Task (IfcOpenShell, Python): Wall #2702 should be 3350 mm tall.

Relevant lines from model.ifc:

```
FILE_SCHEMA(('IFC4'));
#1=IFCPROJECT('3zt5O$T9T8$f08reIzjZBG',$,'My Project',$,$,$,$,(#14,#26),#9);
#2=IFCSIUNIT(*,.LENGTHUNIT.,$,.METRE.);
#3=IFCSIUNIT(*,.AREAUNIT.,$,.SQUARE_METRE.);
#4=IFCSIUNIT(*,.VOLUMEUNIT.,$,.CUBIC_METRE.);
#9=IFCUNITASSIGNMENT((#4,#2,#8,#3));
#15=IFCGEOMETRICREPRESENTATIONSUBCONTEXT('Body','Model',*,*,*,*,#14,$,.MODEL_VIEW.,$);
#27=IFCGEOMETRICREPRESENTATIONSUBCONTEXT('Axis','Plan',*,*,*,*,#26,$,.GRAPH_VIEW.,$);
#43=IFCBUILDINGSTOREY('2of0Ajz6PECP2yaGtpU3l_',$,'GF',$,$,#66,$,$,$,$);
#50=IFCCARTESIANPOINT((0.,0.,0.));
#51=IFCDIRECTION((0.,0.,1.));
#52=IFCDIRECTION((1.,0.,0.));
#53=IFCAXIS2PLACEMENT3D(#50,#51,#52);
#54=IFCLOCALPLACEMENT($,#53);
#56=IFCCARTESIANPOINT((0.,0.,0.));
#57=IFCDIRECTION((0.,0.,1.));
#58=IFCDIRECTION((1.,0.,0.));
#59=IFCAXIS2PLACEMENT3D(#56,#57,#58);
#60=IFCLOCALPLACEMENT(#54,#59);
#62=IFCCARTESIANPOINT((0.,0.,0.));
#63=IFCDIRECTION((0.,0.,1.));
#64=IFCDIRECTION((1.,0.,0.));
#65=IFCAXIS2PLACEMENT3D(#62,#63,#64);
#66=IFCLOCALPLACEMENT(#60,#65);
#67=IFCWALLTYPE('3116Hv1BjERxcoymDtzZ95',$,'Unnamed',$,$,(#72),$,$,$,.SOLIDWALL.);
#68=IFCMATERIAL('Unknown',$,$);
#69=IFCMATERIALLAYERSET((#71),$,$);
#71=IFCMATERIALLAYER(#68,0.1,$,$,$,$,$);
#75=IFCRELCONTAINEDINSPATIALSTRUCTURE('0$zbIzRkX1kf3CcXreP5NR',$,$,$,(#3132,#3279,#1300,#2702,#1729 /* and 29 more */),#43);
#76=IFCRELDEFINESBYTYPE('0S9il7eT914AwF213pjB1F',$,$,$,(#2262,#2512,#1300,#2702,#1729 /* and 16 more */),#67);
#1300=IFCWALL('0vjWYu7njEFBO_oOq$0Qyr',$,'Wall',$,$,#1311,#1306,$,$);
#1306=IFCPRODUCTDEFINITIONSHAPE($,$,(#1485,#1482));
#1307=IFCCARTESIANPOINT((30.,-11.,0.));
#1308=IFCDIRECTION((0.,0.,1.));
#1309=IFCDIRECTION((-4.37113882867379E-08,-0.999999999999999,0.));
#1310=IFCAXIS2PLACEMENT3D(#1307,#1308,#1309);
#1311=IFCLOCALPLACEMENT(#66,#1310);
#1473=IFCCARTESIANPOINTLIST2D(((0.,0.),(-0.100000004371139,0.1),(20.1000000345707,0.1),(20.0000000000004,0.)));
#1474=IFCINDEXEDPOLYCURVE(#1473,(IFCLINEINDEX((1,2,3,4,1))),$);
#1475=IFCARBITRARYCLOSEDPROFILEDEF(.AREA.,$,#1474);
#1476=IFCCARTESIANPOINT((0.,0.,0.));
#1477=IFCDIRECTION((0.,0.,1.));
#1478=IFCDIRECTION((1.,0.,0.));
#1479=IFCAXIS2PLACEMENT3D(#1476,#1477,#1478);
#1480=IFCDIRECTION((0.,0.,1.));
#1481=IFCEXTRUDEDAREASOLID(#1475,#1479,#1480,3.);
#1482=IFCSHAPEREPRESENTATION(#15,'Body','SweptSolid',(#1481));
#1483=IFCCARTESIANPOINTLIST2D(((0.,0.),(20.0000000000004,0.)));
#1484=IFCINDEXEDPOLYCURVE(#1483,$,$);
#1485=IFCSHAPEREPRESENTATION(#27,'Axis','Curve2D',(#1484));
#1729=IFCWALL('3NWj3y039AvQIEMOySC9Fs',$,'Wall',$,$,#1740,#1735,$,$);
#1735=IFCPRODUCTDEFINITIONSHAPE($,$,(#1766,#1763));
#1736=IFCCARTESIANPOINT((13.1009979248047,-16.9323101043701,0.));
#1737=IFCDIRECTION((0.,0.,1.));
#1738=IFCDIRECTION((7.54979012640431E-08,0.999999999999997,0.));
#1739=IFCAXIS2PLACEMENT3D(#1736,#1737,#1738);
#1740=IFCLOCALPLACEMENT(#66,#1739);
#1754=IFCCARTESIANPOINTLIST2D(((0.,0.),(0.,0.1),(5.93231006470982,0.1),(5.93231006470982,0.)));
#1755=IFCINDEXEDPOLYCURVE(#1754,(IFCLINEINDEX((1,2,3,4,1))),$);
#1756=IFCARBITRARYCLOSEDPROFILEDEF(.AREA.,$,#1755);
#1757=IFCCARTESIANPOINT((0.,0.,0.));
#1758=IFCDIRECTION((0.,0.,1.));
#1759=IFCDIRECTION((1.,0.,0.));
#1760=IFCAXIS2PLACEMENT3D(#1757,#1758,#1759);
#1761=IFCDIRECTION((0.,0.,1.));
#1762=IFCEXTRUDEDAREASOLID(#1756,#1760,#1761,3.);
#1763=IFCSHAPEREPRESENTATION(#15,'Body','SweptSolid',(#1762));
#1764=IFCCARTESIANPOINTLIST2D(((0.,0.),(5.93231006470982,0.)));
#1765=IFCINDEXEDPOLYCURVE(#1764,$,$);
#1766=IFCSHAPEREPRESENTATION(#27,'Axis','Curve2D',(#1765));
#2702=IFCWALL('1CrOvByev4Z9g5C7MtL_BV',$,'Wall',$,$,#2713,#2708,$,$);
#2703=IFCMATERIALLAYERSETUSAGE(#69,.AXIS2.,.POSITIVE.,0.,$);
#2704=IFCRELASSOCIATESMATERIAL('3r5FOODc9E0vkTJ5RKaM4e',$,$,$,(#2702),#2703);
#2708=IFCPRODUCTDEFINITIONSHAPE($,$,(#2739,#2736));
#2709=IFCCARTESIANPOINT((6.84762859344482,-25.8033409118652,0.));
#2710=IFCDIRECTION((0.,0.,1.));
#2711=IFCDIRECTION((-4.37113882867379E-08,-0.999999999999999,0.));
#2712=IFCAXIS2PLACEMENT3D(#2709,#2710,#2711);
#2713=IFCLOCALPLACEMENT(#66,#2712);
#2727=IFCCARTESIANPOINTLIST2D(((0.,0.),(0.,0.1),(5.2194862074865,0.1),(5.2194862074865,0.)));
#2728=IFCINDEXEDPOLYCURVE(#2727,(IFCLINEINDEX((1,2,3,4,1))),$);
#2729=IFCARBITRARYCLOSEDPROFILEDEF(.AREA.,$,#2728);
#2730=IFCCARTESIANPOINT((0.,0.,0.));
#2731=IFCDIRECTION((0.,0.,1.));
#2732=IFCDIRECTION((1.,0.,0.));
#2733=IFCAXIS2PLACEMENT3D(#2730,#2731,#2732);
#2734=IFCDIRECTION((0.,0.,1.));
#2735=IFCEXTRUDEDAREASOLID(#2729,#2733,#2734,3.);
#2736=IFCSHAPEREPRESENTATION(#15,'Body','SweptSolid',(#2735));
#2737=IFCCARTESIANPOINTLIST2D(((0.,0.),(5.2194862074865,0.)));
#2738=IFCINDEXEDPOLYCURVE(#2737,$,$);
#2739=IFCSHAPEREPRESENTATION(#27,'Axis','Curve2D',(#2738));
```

```python
import ifcopenshell
import ifcopenshell.geom
import ifcopenshell.util.representation
import ifcopenshell.util.shape

model = ifcopenshell.open("model.ifc")
settings = ifcopenshell.geom.settings()


def volume(element):
    """Net volume in cubic metres, openings subtracted."""
    shape = ifcopenshell.geom.create_shape(settings, element)
    return ifcopenshell.util.shape.get_volume(shape.geometry)


wall = model.by_guid("1CrOvByev4Z9g5C7MtL_BV")
before = volume(wall)

body = ifcopenshell.util.representation.get_representation(wall, "Model", "Body")
solid = body.Items[0]
old_height = solid.Depth
solid.Depth = 3.35
after = volume(wall)

print(f"height {old_height:g} -> {solid.Depth:g}, volume {before:.3f} -> {after:.3f} m3")

model.write("model_updated.ifc")
```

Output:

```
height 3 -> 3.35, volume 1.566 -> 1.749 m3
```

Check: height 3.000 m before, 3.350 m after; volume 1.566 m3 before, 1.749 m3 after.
